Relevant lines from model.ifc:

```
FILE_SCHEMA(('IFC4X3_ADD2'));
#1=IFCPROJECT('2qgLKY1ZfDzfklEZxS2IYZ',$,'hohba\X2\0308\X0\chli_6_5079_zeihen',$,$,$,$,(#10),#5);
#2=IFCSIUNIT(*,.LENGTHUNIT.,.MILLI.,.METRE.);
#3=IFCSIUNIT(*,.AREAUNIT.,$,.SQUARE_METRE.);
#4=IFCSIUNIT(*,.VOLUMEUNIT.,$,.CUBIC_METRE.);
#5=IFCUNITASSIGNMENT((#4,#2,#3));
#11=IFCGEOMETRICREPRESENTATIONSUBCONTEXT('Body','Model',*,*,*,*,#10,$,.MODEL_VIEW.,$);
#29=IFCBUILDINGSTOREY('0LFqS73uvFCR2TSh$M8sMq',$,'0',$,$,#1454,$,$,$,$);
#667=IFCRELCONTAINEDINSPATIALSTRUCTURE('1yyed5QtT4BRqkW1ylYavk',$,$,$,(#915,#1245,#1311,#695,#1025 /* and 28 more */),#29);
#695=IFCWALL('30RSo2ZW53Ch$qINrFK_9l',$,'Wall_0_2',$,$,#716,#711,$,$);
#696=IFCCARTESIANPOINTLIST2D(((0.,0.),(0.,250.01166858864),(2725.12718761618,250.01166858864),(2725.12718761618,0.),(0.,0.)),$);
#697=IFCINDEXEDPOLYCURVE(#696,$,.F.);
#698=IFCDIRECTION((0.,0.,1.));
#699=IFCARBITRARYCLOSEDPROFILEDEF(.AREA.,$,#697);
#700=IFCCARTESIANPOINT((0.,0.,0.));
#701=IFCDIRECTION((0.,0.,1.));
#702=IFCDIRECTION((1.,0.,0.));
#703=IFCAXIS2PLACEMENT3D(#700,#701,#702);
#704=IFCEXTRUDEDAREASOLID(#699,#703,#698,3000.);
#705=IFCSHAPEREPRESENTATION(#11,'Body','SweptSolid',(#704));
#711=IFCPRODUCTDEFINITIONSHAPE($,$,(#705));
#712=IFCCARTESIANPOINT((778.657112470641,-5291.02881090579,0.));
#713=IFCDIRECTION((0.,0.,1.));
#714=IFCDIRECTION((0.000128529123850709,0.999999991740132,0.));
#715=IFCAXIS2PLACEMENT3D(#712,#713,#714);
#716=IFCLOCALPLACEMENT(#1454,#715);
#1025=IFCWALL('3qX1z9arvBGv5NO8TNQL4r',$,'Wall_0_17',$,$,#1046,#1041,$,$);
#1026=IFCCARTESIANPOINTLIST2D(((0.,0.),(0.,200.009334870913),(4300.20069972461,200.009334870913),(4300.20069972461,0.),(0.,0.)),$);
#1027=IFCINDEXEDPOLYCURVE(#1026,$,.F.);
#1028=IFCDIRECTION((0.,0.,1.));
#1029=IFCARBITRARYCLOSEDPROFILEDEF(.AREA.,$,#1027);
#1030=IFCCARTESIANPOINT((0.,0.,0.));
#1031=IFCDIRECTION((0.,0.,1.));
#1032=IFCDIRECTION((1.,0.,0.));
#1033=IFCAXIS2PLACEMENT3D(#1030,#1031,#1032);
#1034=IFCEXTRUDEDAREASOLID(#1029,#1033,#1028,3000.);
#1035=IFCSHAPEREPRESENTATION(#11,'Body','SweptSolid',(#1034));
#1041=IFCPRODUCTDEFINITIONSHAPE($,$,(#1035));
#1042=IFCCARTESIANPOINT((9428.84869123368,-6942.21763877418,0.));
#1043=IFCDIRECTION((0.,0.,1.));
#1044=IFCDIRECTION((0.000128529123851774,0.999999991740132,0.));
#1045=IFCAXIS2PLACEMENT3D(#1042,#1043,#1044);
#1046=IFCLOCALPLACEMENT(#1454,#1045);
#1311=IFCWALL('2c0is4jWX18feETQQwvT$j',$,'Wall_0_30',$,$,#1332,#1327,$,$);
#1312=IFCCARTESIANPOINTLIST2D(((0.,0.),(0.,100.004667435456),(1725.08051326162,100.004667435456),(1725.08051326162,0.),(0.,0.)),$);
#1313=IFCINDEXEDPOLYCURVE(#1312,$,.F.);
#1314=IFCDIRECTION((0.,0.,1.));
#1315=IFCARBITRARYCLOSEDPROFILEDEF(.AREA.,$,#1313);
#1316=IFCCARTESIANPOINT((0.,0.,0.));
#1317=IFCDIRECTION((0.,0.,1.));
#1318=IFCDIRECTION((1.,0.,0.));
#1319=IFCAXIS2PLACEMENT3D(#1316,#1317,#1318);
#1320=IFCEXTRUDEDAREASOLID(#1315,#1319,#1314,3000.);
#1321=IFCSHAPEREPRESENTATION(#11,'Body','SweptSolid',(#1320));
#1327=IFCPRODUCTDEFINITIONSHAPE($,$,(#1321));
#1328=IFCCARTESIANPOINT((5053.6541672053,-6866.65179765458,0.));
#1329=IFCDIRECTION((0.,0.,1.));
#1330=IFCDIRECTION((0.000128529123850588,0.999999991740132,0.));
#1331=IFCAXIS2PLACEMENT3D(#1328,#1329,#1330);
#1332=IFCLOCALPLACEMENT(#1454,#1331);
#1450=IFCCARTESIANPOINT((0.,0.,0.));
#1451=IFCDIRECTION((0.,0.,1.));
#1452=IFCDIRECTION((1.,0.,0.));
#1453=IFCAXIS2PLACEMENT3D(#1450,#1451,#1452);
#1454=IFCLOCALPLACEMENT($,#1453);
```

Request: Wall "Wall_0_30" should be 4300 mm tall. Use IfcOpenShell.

```python
import ifcopenshell
import ifcopenshell.geom
import ifcopenshell.util.representation
import ifcopenshell.util.shape
import ifcopenshell.util.unit

model = ifcopenshell.open("model.ifc")
unit_scale = ifcopenshell.util.unit.calculate_unit_scale(model)
settings = ifcopenshell.geom.settings()


def volume(element):
    """Net volume in cubic metres, openings subtracted."""
    shape = ifcopenshell.geom.create_shape(settings, element)
    return ifcopenshell.util.shape.get_volume(shape.geometry)


wall = model.by_id(1311)
before = volume(wall)

body = ifcopenshell.util.representation.get_representation(wall, "Model", "Body")
solid = body.Items[0]
old_height = solid.Depth
solid.Depth = 4.3 / unit_scale
after = volume(wall)

print(f"height {old_height:g} -> {solid.Depth:g}, volume {before:.3f} -> {after:.3f} m3")

model.write("model_edited.ifc")
```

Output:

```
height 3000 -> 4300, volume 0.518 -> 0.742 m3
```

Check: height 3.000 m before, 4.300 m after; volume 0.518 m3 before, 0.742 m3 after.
